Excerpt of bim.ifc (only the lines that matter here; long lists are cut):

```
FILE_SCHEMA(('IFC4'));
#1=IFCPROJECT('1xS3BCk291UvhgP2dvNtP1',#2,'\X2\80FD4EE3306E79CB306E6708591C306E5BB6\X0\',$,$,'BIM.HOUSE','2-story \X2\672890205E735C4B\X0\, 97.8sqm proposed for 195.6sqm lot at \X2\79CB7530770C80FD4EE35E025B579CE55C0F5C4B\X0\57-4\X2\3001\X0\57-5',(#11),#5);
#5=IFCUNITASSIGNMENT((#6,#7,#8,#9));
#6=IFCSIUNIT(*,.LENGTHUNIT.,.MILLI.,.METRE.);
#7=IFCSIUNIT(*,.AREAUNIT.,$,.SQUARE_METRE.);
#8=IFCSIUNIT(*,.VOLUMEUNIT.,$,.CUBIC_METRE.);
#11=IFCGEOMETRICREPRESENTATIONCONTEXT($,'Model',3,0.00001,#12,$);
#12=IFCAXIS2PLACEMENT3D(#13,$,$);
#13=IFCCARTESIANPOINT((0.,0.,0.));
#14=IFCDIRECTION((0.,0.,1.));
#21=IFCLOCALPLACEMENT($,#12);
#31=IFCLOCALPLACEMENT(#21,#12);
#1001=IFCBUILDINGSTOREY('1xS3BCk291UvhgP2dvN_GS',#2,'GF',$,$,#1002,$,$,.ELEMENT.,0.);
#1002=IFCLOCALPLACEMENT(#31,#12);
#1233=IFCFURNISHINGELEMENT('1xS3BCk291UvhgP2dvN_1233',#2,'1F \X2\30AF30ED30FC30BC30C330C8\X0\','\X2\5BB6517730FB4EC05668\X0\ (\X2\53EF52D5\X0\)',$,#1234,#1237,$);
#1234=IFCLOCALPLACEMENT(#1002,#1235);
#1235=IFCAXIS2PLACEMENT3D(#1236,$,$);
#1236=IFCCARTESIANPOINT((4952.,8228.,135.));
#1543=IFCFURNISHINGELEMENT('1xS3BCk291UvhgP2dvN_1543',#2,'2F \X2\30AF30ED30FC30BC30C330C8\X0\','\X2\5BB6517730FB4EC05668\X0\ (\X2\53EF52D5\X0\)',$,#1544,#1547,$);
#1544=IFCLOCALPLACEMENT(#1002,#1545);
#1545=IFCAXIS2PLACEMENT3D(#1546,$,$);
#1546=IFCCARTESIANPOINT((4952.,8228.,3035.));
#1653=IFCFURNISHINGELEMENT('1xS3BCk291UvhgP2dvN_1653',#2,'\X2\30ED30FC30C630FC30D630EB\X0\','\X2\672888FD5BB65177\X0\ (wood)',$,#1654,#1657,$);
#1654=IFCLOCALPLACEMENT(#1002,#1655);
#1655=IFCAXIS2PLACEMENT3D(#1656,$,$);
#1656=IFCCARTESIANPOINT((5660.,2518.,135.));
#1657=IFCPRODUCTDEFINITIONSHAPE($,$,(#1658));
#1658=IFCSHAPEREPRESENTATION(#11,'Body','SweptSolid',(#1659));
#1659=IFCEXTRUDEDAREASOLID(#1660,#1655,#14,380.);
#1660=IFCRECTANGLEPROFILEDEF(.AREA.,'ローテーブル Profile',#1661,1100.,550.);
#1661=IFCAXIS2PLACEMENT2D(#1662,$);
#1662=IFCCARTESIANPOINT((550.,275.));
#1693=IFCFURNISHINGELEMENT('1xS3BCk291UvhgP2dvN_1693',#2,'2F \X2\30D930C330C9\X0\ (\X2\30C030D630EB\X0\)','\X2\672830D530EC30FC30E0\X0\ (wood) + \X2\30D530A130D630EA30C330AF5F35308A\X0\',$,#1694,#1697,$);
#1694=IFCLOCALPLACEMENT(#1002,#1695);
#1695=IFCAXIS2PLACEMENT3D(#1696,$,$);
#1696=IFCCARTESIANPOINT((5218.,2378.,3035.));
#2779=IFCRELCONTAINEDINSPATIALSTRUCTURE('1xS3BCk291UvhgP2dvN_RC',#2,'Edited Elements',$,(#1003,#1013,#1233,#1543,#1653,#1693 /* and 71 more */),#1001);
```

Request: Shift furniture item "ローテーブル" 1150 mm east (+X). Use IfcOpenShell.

```python
import ifcopenshell
import ifcopenshell.api.geometry
import ifcopenshell.util.placement

model = ifcopenshell.open("bim.ifc")

item = model.by_guid("1xS3BCk291UvhgP2dvN_1653")
matrix = ifcopenshell.util.placement.get_local_placement(item.ObjectPlacement)
matrix[0, 3] += 1150.0
ifcopenshell.api.geometry.edit_object_placement(model, product=item, matrix=matrix, is_si=False)

print(ifcopenshell.util.placement.get_local_placement(item.ObjectPlacement).round(3) + 0.0)

model.write("bim_v2.ifc")
```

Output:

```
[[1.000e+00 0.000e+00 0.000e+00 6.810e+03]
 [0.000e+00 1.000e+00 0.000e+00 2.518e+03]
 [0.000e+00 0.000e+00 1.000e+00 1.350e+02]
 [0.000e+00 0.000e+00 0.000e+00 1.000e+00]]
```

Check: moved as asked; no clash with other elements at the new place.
